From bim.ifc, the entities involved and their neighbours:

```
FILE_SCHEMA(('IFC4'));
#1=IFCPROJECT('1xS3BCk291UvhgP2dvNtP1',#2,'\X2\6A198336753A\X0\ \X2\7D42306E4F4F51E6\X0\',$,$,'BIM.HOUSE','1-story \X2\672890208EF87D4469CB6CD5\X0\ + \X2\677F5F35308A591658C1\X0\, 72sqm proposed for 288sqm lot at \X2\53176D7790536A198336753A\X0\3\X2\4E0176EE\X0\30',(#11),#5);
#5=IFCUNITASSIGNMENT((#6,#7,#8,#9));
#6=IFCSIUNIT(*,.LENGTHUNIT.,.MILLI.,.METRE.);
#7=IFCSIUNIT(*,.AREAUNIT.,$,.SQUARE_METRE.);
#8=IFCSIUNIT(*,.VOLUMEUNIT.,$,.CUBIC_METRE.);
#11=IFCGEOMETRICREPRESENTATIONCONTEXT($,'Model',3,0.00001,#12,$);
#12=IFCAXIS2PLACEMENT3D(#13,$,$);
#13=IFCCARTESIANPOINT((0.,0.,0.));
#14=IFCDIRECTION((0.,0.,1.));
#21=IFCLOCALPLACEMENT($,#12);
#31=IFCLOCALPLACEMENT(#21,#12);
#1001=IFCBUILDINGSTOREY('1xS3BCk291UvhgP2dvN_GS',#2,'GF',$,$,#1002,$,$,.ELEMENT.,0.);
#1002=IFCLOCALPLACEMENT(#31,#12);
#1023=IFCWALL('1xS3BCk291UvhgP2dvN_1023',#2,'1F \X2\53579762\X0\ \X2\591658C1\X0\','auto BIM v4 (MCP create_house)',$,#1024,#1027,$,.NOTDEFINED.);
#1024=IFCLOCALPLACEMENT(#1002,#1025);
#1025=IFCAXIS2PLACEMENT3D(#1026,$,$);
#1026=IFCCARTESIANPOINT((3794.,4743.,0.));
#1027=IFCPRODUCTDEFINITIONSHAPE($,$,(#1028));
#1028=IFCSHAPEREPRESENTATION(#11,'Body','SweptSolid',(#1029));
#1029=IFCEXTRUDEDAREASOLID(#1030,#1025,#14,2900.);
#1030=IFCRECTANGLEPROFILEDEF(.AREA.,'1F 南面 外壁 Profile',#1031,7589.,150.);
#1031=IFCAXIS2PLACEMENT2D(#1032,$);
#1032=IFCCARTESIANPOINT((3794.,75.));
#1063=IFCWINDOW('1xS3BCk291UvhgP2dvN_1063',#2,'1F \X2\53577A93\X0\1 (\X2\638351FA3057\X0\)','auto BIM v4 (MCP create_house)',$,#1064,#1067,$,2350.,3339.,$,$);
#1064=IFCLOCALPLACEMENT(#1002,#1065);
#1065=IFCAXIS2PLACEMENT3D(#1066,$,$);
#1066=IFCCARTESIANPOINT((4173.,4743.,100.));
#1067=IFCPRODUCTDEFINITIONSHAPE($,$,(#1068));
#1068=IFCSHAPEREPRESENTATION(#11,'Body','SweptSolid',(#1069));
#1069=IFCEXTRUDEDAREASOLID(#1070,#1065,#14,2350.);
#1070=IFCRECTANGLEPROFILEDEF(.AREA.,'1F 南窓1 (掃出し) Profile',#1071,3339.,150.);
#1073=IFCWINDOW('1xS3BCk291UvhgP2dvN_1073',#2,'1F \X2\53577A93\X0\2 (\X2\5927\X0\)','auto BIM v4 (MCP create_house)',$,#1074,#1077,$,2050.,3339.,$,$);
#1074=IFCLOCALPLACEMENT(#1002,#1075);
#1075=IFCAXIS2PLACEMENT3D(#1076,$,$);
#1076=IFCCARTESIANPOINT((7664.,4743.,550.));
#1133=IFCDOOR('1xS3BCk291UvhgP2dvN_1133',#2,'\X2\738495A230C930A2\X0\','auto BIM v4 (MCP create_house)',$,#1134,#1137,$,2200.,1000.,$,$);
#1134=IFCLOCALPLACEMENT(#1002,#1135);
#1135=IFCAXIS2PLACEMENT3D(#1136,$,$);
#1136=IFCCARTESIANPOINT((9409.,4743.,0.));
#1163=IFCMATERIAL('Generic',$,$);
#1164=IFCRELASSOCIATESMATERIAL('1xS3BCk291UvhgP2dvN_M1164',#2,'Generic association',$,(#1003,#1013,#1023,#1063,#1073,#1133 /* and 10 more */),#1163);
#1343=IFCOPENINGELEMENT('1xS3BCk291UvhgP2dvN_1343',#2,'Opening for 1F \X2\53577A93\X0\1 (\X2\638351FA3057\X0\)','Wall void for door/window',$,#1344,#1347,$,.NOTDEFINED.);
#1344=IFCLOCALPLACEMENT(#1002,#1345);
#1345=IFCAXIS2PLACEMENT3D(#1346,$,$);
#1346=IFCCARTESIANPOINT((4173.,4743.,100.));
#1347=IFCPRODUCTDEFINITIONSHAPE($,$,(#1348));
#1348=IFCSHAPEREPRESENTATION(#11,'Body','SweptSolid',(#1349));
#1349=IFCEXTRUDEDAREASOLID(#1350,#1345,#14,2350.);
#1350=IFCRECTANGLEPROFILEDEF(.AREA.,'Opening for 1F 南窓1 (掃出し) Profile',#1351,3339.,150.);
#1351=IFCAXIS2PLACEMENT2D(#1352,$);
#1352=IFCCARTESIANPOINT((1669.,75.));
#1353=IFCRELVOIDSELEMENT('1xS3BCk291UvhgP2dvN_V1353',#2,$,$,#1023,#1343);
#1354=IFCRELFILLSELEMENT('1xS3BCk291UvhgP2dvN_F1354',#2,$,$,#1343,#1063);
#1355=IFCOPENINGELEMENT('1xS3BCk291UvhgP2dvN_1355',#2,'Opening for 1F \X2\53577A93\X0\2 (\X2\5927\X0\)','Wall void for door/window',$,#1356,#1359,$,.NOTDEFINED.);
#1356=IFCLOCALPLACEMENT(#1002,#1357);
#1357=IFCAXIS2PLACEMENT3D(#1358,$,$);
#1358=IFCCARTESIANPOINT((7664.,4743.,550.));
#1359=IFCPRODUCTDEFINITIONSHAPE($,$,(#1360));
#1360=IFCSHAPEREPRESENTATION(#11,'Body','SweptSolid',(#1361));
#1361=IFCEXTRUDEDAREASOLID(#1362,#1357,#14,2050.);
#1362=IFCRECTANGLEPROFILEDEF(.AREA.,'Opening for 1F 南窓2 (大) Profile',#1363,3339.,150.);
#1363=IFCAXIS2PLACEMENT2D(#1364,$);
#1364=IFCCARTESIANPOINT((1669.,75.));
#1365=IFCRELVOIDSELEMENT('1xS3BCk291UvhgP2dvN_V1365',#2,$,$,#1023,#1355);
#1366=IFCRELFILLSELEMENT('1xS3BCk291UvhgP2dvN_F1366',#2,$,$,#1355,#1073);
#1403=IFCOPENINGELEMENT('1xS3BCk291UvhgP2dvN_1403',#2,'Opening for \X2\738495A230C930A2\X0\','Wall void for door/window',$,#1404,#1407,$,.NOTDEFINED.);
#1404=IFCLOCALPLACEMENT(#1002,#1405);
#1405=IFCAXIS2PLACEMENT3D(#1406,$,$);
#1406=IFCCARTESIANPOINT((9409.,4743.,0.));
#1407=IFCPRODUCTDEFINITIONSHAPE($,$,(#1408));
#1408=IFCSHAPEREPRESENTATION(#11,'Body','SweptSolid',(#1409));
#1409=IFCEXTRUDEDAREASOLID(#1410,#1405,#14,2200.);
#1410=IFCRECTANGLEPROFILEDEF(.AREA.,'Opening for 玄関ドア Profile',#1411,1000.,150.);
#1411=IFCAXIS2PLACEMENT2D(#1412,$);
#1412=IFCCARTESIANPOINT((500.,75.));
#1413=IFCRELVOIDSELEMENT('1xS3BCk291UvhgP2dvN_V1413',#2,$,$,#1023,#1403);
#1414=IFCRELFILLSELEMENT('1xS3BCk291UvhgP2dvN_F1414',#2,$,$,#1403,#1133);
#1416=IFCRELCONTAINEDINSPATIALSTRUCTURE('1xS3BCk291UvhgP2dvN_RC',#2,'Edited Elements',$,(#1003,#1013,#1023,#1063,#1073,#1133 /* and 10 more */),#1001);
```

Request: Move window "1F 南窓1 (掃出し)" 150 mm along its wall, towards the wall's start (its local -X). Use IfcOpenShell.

```python
import ifcopenshell
import ifcopenshell.api.geometry
import ifcopenshell.util.placement
import ifcopenshell.util.unit

model = ifcopenshell.open("bim.ifc")
unit_scale = ifcopenshell.util.unit.calculate_unit_scale(model)

window = model.by_guid("1xS3BCk291UvhgP2dvN_1063")
opening = window.FillsVoids[0].RelatingOpeningElement
wall = opening.VoidsElements[0].RelatingBuildingElement

wall_matrix = ifcopenshell.util.placement.get_local_placement(wall.ObjectPlacement)
shift = wall_matrix[:3, 0] * -0.15 / unit_scale
before = ifcopenshell.util.placement.get_local_placement(window.ObjectPlacement)[:3, 3].copy()

# The window is not placed relative to its opening, so move both.
for product in (opening, window):
    matrix = ifcopenshell.util.placement.get_local_placement(product.ObjectPlacement)
    matrix[:3, 3] += shift
    ifcopenshell.api.geometry.edit_object_placement(model, product=product, matrix=matrix, is_si=False)

after = ifcopenshell.util.placement.get_local_placement(window.ObjectPlacement)[:3, 3]
print("window moved by", (after - before).round(3) + 0.0)

model.write("bim-out.ifc")
```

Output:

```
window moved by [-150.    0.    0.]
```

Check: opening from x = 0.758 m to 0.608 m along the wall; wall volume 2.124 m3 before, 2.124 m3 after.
